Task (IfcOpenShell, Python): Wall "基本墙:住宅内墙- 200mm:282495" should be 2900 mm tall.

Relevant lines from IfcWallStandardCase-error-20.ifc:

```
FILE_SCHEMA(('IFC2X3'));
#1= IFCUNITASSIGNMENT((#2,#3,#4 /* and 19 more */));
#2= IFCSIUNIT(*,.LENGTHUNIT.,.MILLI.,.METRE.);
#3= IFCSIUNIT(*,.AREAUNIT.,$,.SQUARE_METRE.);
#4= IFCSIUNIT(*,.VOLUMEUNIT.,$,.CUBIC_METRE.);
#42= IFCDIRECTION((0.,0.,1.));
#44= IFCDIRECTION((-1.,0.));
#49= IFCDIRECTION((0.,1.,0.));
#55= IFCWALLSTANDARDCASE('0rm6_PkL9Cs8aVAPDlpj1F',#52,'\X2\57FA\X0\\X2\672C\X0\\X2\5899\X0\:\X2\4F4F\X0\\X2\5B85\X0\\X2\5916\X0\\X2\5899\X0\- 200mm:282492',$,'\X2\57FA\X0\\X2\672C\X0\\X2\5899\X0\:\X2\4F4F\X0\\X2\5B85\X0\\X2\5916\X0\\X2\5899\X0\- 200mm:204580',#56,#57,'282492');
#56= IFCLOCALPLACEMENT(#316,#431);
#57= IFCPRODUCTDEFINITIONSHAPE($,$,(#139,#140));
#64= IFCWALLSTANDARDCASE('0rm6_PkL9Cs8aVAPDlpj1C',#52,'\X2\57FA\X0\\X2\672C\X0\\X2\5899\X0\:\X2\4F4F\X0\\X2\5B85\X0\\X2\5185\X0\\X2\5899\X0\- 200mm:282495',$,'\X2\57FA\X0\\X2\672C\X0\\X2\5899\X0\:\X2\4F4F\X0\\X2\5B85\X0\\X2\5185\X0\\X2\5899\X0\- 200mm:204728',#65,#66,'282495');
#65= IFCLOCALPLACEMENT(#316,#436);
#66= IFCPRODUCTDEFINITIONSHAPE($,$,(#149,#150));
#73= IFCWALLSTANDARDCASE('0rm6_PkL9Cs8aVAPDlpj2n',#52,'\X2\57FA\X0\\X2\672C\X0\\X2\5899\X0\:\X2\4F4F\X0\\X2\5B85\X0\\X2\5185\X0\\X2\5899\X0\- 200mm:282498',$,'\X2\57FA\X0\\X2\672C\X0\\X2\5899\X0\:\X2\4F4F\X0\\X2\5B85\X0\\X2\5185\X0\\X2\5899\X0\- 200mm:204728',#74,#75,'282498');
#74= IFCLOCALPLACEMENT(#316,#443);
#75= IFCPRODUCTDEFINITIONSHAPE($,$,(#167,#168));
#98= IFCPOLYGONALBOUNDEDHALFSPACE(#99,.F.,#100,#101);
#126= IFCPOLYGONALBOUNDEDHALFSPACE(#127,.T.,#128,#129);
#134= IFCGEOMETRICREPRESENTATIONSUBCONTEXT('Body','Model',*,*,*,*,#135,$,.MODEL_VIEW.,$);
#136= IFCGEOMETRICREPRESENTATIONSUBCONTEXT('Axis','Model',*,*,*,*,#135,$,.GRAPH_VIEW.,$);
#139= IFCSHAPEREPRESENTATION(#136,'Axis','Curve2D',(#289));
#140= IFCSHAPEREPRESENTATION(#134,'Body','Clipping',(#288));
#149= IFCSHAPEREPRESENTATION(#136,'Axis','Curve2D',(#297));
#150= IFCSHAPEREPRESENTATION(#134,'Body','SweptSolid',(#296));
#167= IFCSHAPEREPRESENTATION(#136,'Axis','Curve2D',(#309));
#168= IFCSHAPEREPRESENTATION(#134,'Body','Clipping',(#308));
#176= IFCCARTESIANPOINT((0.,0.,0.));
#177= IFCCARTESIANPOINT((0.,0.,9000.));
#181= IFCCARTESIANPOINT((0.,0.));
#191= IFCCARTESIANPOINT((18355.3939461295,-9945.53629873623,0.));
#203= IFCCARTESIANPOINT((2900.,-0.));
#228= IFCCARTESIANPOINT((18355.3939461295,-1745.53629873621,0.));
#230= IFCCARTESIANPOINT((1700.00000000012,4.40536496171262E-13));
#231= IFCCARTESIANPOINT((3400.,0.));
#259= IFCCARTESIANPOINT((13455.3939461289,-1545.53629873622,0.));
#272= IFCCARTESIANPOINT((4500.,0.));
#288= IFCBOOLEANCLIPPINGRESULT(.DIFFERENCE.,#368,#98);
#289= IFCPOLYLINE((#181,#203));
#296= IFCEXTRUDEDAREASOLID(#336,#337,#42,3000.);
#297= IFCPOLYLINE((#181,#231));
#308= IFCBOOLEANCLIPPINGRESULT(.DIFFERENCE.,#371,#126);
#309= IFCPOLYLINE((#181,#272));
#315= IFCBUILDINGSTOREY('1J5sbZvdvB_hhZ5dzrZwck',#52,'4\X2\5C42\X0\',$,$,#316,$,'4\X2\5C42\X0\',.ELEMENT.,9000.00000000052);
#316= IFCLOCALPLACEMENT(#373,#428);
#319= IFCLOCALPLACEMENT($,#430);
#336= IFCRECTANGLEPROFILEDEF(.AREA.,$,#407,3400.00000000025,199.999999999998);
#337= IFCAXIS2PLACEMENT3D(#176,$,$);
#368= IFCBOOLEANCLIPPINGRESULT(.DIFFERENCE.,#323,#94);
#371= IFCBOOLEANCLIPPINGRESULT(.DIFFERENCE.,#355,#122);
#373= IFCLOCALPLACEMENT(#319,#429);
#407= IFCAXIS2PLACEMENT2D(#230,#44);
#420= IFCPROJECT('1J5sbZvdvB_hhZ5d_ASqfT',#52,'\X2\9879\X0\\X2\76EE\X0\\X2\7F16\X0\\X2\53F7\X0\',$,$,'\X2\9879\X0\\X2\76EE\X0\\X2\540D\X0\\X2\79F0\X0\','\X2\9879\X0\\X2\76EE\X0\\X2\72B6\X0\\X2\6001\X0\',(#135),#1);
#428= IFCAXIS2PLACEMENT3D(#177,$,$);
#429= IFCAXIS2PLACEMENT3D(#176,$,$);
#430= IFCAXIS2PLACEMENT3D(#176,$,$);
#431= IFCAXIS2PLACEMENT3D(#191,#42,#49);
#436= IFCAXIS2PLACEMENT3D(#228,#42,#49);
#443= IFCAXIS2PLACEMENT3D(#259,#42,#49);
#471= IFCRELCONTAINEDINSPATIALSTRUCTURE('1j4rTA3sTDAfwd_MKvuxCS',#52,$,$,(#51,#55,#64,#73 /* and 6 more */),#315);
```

```python
import ifcopenshell
import ifcopenshell.geom
import ifcopenshell.util.representation
import ifcopenshell.util.shape

model = ifcopenshell.open("IfcWallStandardCase-error-20.ifc")
settings = ifcopenshell.geom.settings()


def volume(element):
    """Net volume in cubic metres, openings subtracted."""
    shape = ifcopenshell.geom.create_shape(settings, element)
    return ifcopenshell.util.shape.get_volume(shape.geometry)


wall = model.by_guid("0rm6_PkL9Cs8aVAPDlpj1C")
before = volume(wall)

body = ifcopenshell.util.representation.get_representation(wall, "Model", "Body")
solid = body.Items[0]
old_height = solid.Depth
solid.Depth = 2900.0
after = volume(wall)

print(f"height {old_height:g} -> {solid.Depth:g}, volume {before:.3f} -> {after:.3f} m3")

model.write("IfcWallStandardCase-error-20_v2.ifc")
```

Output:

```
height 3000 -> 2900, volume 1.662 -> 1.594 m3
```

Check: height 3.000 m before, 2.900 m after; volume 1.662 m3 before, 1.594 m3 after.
